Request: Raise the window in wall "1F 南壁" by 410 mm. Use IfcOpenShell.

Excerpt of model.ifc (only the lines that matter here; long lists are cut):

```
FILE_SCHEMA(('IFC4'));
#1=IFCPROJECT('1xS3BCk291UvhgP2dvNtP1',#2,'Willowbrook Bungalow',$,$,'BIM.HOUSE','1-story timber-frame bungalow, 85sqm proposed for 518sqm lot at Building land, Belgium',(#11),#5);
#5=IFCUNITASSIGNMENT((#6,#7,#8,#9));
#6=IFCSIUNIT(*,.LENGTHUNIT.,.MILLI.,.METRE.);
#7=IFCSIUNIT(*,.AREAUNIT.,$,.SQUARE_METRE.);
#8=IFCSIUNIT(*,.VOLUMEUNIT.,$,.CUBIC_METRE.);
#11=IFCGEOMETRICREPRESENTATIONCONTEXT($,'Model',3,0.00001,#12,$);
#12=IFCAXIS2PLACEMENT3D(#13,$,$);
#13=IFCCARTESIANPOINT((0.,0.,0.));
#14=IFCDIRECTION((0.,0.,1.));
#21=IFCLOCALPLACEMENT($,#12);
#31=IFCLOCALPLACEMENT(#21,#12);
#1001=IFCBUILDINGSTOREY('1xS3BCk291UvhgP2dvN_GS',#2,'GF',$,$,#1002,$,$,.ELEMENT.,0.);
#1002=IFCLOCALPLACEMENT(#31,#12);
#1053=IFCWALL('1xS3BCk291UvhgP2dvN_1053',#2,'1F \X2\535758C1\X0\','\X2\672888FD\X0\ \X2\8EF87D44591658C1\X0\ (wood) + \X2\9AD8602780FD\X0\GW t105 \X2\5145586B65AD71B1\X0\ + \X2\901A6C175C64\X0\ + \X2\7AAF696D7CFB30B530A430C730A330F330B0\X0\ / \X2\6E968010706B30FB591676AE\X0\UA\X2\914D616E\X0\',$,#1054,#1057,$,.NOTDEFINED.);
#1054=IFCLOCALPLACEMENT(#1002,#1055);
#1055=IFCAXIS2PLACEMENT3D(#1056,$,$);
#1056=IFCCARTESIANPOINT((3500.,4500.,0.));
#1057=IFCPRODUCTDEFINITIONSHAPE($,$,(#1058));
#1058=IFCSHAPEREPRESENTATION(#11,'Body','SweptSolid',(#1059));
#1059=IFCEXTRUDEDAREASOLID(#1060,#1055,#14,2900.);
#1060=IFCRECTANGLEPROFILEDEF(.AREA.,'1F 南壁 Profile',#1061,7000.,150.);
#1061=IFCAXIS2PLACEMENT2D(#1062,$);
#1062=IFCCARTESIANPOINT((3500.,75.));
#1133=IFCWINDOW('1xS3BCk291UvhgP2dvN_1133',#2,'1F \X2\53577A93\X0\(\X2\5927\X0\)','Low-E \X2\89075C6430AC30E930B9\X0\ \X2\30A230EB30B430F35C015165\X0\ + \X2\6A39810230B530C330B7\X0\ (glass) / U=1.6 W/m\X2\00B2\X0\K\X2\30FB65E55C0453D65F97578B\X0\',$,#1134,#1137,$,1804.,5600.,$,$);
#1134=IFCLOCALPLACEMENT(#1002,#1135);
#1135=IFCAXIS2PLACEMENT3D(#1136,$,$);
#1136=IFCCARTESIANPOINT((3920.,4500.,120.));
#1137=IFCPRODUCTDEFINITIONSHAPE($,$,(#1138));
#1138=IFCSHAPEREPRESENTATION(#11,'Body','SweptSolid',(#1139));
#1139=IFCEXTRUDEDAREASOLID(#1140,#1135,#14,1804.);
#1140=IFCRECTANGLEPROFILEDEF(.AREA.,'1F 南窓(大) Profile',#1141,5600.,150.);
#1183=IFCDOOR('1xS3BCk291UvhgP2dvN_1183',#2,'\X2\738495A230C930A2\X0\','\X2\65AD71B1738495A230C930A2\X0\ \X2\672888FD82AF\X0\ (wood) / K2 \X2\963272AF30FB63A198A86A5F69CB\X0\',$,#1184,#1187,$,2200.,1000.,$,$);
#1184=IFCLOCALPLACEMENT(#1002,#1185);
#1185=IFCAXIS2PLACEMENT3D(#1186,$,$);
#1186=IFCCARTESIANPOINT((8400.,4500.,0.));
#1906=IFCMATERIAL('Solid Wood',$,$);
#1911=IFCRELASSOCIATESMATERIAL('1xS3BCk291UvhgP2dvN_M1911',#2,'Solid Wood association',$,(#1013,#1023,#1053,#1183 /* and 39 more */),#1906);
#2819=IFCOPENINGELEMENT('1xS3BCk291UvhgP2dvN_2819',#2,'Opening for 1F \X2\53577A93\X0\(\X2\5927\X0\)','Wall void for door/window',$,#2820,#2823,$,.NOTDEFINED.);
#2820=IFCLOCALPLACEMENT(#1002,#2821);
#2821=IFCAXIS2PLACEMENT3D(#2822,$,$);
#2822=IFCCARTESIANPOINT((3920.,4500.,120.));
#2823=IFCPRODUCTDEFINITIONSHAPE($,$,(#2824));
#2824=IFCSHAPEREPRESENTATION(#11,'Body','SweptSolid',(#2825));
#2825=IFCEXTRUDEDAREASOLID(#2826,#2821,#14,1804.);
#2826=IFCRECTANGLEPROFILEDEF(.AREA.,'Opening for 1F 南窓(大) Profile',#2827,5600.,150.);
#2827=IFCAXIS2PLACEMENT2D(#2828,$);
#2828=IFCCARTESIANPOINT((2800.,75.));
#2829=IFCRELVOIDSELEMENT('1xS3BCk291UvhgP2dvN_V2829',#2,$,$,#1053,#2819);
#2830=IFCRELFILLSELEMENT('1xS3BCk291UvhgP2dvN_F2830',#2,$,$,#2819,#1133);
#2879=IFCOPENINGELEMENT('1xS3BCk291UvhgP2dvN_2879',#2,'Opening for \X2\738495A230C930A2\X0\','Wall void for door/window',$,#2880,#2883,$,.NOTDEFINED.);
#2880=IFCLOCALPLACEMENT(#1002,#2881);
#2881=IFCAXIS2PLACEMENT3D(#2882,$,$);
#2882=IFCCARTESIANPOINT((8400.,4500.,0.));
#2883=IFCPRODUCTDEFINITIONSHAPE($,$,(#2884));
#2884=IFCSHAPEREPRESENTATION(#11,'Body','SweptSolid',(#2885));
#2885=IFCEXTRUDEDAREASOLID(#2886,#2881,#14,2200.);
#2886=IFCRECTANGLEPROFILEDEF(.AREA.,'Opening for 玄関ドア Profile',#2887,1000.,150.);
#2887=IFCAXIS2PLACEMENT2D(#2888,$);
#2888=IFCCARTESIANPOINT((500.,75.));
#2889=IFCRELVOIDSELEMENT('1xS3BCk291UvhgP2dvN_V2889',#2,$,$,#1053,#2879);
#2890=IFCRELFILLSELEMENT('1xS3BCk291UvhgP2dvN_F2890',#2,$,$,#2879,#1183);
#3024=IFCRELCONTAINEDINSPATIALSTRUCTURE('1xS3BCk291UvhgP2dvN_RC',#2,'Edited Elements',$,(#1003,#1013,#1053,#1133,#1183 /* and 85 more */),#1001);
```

```python
import numpy as np
import ifcopenshell
import ifcopenshell.api.geometry
import ifcopenshell.util.placement
import ifcopenshell.util.unit

model = ifcopenshell.open("model.ifc")
unit_scale = ifcopenshell.util.unit.calculate_unit_scale(model)

window = model.by_guid("1xS3BCk291UvhgP2dvN_1133")
opening = window.FillsVoids[0].RelatingOpeningElement
dz = 410.0

shift = np.array([0.0, 0.0, dz])
# The window is not placed relative to its opening, so move both.
for product in (opening, window):
    matrix = ifcopenshell.util.placement.get_local_placement(product.ObjectPlacement)
    matrix[:3, 3] += shift
    ifcopenshell.api.geometry.edit_object_placement(model, product=product, matrix=matrix, is_si=False)

print(f"moved by {dz * unit_scale:+.3f} m")

model.write("model_updated.ifc")
```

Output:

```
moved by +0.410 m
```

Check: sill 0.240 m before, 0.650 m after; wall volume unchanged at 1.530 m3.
